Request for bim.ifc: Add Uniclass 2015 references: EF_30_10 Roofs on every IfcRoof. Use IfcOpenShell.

First a look at what the model holds.

```python
import ifcopenshell

model = ifcopenshell.open("bim.ifc")
print(model.schema)
print("classifications:", [c.Name for c in model.by_type("IfcClassification")])
for ifc_class in ("IfcDoor", "IfcRoof", "IfcStair", "IfcWall", "IfcWindow"):
    print(ifc_class, len(model.by_type(ifc_class)))
```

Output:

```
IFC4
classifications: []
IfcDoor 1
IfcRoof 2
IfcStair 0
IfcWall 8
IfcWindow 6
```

```python
import ifcopenshell
import ifcopenshell.api.classification

model = ifcopenshell.open("bim.ifc")

system = ifcopenshell.api.classification.add_classification(model, classification="Uniclass 2015")

codes = {
    "IfcRoof": ("EF_30_10", "Roofs"),
}
for ifc_class, (code, name) in codes.items():
    products = model.by_type(ifc_class)
    ifcopenshell.api.classification.add_reference(
        model, products=products, classification=system, identification=code, name=name
    )
    print(code, len(products))

model.write("bim_rev.ifc")
```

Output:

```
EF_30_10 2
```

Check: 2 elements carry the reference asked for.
